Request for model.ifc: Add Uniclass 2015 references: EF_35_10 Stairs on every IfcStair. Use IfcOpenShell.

First a look at what the model holds.

```python
import ifcopenshell

model = ifcopenshell.open("model.ifc")
print(model.schema)
print("classifications:", [c.Name for c in model.by_type("IfcClassification")])
for ifc_class in ("IfcDoor", "IfcRoof", "IfcStair", "IfcWall", "IfcWindow"):
    print(ifc_class, len(model.by_type(ifc_class)))
```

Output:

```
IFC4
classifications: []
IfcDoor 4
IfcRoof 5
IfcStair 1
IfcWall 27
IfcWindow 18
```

```python
import ifcopenshell
import ifcopenshell.api.classification

model = ifcopenshell.open("model.ifc")

system = ifcopenshell.api.classification.add_classification(model, classification="Uniclass 2015")

codes = {
    "IfcStair": ("EF_35_10", "Stairs"),
}
for ifc_class, (code, name) in codes.items():
    products = model.by_type(ifc_class)
    ifcopenshell.api.classification.add_reference(
        model, products=products, classification=system, identification=code, name=name
    )
    print(code, len(products))

model.write("model_v2.ifc")
```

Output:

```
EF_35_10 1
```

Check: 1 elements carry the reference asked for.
